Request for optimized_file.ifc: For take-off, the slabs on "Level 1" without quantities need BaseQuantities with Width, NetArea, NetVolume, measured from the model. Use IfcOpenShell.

First a look at what the model holds.

```python
import ifcopenshell
import ifcopenshell.util.element
import ifcopenshell.util.unit

model = ifcopenshell.open("optimized_file.ifc")
print(model.schema)
for unit_type in ("LENGTHUNIT", "AREAUNIT", "VOLUMEUNIT"):
    print(unit_type, ifcopenshell.util.unit.calculate_unit_scale(model, unit_type))
storey = next(s for s in model.by_type("IfcBuildingStorey") if s.Name == "Level 1")
slabs = [e for e in ifcopenshell.util.element.get_decomposition(storey) if e.is_a("IfcSlab")]
for e in sorted(slabs, key=lambda e: e.id()):
    print(e.id(), e.is_a(), e.Name, list(ifcopenshell.util.element.get_psets(e, qtos_only=True)), sep=" | ")
```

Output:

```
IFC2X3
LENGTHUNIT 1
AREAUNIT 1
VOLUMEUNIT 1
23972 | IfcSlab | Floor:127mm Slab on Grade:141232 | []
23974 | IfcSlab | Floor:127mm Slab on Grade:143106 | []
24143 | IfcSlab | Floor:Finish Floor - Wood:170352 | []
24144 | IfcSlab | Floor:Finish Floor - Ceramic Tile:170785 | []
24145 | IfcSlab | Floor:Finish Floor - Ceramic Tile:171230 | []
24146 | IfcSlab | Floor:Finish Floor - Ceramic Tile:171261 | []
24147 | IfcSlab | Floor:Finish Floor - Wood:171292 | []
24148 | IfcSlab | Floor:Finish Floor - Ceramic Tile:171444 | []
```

```python
import ifcopenshell
import ifcopenshell.api.pset
import ifcopenshell.geom
import ifcopenshell.util.element
import ifcopenshell.util.shape
import ifcopenshell.util.unit

model = ifcopenshell.open("optimized_file.ifc")
unit_scale = ifcopenshell.util.unit.calculate_unit_scale(model)
area_scale = ifcopenshell.util.unit.calculate_unit_scale(model, "AREAUNIT")
volume_scale = ifcopenshell.util.unit.calculate_unit_scale(model, "VOLUMEUNIT")
settings = ifcopenshell.geom.settings()

storey = next(s for s in model.by_type("IfcBuildingStorey") if s.Name == "Level 1")
slabs = [e for e in ifcopenshell.util.element.get_decomposition(storey) if e.is_a("IfcSlab")]

for e in sorted(slabs, key=lambda e: e.id()):
    if ifcopenshell.util.element.get_psets(e, qtos_only=True, should_inherit=False):
        continue
    # Geometry comes back in metres, in the element's own axes.
    shape = ifcopenshell.geom.create_shape(settings, e)
    values = {
        "Width": ifcopenshell.util.shape.get_z(shape.geometry) / unit_scale,
        "NetArea": ifcopenshell.util.shape.get_footprint_area(shape.geometry) / area_scale,
        "NetVolume": ifcopenshell.util.shape.get_volume(shape.geometry) / volume_scale,
    }
    qto = ifcopenshell.api.pset.add_qto(model, product=e, name="BaseQuantities")
    ifcopenshell.api.pset.edit_qto(model, qto=qto, properties=values)
    print(e.id(), {k: round(v, 3) for k, v in values.items()})

model.write("optimized_file_updated.ifc")
```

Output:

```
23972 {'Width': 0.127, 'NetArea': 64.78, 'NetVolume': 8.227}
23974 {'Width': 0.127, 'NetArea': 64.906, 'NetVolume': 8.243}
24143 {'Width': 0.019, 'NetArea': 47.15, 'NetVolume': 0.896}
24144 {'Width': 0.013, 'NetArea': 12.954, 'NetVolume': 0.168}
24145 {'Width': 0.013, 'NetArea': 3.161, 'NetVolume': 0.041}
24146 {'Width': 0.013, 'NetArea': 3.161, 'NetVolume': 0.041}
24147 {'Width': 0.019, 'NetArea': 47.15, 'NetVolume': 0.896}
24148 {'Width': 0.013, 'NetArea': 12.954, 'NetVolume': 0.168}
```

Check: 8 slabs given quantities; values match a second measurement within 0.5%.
